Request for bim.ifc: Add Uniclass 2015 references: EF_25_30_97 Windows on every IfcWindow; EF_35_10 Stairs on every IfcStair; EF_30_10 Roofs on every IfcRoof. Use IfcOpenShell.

First a look at what the model holds.

```python
import ifcopenshell

model = ifcopenshell.open("bim.ifc")
print(model.schema)
print("classifications:", [c.Name for c in model.by_type("IfcClassification")])
for ifc_class in ("IfcDoor", "IfcRoof", "IfcStair", "IfcWall", "IfcWindow"):
    print(ifc_class, len(model.by_type(ifc_class)))
```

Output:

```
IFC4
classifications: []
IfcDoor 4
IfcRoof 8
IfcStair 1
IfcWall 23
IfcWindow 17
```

```python
import ifcopenshell
import ifcopenshell.api.classification

model = ifcopenshell.open("bim.ifc")

system = ifcopenshell.api.classification.add_classification(model, classification="Uniclass 2015")

codes = {
    "IfcWindow": ("EF_25_30_97", "Windows"),
    "IfcStair": ("EF_35_10", "Stairs"),
    "IfcRoof": ("EF_30_10", "Roofs"),
}
for ifc_class, (code, name) in codes.items():
    products = model.by_type(ifc_class)
    ifcopenshell.api.classification.add_reference(
        model, products=products, classification=system, identification=code, name=name
    )
    print(code, len(products))

model.write("bim-out.ifc")
```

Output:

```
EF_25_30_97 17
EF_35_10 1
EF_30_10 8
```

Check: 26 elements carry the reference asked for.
